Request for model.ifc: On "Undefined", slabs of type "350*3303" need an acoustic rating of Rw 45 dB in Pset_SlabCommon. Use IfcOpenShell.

First a look at what the model holds.

```python
import ifcopenshell
import ifcopenshell.util.element

model = ifcopenshell.open("model.ifc")
print(model.schema)
storey = next(s for s in model.by_type("IfcBuildingStorey") if s.Name == "Undefined")
slabs = [e for e in ifcopenshell.util.element.get_decomposition(storey) if e.is_a("IfcSlab")]
seen = {}
for e in slabs:
    element_type = ifcopenshell.util.element.get_type(e)
    key = (element_type.Name if element_type != e and element_type else None, ifcopenshell.util.element.get_pset(e, "Pset_SlabCommon", "AcousticRating"))
    seen[key] = seen.get(key, 0) + 1
for (name, value), count in sorted(seen.items(), key=str):
    print(count, "x", name, "|", value)
```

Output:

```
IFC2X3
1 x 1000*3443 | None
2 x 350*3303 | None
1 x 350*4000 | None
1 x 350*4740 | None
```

```python
import ifcopenshell
import ifcopenshell.api.pset
import ifcopenshell.util.element

model = ifcopenshell.open("model.ifc")

storey = next(s for s in model.by_type("IfcBuildingStorey") if s.Name == "Undefined")
slabs = [e for e in ifcopenshell.util.element.get_decomposition(storey) if e.is_a("IfcSlab")]

count = 0
for e in slabs:
    element_type = ifcopenshell.util.element.get_type(e)
    if element_type in (None, e) or element_type.Name != "350*3303":
        continue
    found = ifcopenshell.util.element.get_pset(e, "Pset_SlabCommon", should_inherit=False)
    if found:
        pset = model.by_id(found["id"])
        if len(ifcopenshell.util.element.get_elements_by_pset(pset)) > 1:
            pset = ifcopenshell.api.pset.unshare_pset(model, products=[e], pset=pset)[0]
    else:
        pset = ifcopenshell.api.pset.add_pset(model, product=e, name="Pset_SlabCommon")
    ifcopenshell.api.pset.edit_pset(model, pset=pset, properties={"AcousticRating": "Rw 45 dB"})
    count += 1

print(count, "slabs updated")

model.write("model_updated.ifc")
```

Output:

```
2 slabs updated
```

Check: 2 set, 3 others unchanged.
